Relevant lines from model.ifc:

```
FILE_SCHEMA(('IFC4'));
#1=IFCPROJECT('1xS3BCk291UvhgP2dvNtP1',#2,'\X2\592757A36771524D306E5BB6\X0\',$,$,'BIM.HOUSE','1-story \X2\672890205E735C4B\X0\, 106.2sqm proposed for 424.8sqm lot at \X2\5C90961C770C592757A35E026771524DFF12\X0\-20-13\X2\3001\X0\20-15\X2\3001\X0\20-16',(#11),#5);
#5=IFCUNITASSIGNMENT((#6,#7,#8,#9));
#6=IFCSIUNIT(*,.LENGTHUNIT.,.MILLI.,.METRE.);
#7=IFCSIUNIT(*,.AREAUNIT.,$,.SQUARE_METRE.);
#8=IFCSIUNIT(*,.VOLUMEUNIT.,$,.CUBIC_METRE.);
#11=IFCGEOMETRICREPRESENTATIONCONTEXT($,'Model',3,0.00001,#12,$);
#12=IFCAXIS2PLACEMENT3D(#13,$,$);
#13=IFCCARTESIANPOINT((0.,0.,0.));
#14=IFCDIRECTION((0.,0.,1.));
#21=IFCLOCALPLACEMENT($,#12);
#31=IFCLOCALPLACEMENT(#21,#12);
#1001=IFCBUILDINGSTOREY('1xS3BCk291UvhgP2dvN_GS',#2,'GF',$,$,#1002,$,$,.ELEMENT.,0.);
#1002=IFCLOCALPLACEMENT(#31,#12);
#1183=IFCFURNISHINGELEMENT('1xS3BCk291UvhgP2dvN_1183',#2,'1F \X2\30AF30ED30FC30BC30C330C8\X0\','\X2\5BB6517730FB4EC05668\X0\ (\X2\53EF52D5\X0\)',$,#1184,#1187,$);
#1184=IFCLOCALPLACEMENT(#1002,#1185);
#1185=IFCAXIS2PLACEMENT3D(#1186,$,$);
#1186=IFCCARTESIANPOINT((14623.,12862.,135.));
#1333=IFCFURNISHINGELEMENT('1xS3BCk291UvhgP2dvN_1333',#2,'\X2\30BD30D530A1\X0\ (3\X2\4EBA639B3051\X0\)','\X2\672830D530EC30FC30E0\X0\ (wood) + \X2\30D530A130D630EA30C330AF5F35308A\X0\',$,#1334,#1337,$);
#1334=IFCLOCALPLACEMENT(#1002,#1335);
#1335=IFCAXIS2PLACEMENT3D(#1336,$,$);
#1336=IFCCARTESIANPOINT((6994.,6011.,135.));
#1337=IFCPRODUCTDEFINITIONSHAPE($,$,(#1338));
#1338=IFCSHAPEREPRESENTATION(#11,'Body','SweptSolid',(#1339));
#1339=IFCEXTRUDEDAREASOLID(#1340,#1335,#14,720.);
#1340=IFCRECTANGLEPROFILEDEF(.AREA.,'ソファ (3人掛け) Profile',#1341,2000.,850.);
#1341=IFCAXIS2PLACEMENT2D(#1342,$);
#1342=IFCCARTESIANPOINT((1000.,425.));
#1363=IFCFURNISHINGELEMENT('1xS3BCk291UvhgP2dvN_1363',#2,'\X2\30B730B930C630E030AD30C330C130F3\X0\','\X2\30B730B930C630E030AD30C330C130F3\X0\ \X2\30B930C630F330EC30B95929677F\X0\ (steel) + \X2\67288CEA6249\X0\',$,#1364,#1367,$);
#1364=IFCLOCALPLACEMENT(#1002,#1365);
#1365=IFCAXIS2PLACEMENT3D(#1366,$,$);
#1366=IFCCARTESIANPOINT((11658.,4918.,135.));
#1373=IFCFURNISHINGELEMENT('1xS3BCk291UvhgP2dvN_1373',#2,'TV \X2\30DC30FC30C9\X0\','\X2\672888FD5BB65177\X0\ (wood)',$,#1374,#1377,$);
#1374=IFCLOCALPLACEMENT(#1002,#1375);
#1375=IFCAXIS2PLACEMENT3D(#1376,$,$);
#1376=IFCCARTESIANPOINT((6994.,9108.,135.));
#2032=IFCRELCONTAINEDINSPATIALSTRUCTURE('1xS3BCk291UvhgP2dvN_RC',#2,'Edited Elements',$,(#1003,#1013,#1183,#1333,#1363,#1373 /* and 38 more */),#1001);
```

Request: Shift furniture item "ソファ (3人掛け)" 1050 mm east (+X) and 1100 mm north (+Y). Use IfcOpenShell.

```python
import ifcopenshell
import ifcopenshell.api.geometry
import ifcopenshell.util.placement
import ifcopenshell.util.unit

model = ifcopenshell.open("model.ifc")
unit_scale = ifcopenshell.util.unit.calculate_unit_scale(model)

item = model.by_guid("1xS3BCk291UvhgP2dvN_1333")
matrix = ifcopenshell.util.placement.get_local_placement(item.ObjectPlacement)
matrix[0, 3] += 1.05 / unit_scale
matrix[1, 3] += 1.1 / unit_scale
ifcopenshell.api.geometry.edit_object_placement(model, product=item, matrix=matrix, is_si=False)

print(ifcopenshell.util.placement.get_local_placement(item.ObjectPlacement).round(3) + 0.0)

model.write("model_v2.ifc")
```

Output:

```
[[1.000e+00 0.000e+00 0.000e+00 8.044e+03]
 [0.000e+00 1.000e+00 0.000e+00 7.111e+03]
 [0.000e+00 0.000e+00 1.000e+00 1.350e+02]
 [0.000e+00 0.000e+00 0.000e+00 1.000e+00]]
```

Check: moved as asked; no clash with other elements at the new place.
